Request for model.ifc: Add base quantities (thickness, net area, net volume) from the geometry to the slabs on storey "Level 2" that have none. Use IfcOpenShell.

First a look at what the model holds.

```python
import ifcopenshell
import ifcopenshell.util.element
import ifcopenshell.util.unit

model = ifcopenshell.open("model.ifc")
print(model.schema)
for unit_type in ("LENGTHUNIT", "AREAUNIT", "VOLUMEUNIT"):
    print(unit_type, ifcopenshell.util.unit.calculate_unit_scale(model, unit_type))
storey = next(s for s in model.by_type("IfcBuildingStorey") if s.Name == "Level 2")
slabs = [e for e in ifcopenshell.util.element.get_decomposition(storey) if e.is_a("IfcSlab")]
for e in sorted(slabs, key=lambda e: e.id()):
    print(e.id(), e.is_a(), e.Name, list(ifcopenshell.util.element.get_psets(e, qtos_only=True)), sep=" | ")
```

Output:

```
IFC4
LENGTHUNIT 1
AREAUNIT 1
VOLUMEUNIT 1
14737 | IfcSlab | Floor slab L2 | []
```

```python
import ifcopenshell
import ifcopenshell.api.pset
import ifcopenshell.geom
import ifcopenshell.util.element
import ifcopenshell.util.shape
import ifcopenshell.util.unit

model = ifcopenshell.open("model.ifc")
unit_scale = ifcopenshell.util.unit.calculate_unit_scale(model)
area_scale = ifcopenshell.util.unit.calculate_unit_scale(model, "AREAUNIT")
volume_scale = ifcopenshell.util.unit.calculate_unit_scale(model, "VOLUMEUNIT")
settings = ifcopenshell.geom.settings()

storey = next(s for s in model.by_type("IfcBuildingStorey") if s.Name == "Level 2")
slabs = [e for e in ifcopenshell.util.element.get_decomposition(storey) if e.is_a("IfcSlab")]

for e in sorted(slabs, key=lambda e: e.id()):
    if ifcopenshell.util.element.get_psets(e, qtos_only=True, should_inherit=False):
        continue
    # Geometry comes back in metres, in the element's own axes.
    shape = ifcopenshell.geom.create_shape(settings, e)
    values = {
        "Width": ifcopenshell.util.shape.get_z(shape.geometry) / unit_scale,
        "NetArea": ifcopenshell.util.shape.get_footprint_area(shape.geometry) / area_scale,
        "NetVolume": ifcopenshell.util.shape.get_volume(shape.geometry) / volume_scale,
    }
    qto = ifcopenshell.api.pset.add_qto(model, product=e, name="Qto_SlabBaseQuantities")
    ifcopenshell.api.pset.edit_qto(model, qto=qto, properties=values)
    print(e.id(), {k: round(v, 3) for k, v in values.items()})

model.write("model_updated.ifc")
```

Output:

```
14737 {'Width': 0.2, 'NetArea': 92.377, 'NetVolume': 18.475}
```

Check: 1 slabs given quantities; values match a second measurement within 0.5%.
